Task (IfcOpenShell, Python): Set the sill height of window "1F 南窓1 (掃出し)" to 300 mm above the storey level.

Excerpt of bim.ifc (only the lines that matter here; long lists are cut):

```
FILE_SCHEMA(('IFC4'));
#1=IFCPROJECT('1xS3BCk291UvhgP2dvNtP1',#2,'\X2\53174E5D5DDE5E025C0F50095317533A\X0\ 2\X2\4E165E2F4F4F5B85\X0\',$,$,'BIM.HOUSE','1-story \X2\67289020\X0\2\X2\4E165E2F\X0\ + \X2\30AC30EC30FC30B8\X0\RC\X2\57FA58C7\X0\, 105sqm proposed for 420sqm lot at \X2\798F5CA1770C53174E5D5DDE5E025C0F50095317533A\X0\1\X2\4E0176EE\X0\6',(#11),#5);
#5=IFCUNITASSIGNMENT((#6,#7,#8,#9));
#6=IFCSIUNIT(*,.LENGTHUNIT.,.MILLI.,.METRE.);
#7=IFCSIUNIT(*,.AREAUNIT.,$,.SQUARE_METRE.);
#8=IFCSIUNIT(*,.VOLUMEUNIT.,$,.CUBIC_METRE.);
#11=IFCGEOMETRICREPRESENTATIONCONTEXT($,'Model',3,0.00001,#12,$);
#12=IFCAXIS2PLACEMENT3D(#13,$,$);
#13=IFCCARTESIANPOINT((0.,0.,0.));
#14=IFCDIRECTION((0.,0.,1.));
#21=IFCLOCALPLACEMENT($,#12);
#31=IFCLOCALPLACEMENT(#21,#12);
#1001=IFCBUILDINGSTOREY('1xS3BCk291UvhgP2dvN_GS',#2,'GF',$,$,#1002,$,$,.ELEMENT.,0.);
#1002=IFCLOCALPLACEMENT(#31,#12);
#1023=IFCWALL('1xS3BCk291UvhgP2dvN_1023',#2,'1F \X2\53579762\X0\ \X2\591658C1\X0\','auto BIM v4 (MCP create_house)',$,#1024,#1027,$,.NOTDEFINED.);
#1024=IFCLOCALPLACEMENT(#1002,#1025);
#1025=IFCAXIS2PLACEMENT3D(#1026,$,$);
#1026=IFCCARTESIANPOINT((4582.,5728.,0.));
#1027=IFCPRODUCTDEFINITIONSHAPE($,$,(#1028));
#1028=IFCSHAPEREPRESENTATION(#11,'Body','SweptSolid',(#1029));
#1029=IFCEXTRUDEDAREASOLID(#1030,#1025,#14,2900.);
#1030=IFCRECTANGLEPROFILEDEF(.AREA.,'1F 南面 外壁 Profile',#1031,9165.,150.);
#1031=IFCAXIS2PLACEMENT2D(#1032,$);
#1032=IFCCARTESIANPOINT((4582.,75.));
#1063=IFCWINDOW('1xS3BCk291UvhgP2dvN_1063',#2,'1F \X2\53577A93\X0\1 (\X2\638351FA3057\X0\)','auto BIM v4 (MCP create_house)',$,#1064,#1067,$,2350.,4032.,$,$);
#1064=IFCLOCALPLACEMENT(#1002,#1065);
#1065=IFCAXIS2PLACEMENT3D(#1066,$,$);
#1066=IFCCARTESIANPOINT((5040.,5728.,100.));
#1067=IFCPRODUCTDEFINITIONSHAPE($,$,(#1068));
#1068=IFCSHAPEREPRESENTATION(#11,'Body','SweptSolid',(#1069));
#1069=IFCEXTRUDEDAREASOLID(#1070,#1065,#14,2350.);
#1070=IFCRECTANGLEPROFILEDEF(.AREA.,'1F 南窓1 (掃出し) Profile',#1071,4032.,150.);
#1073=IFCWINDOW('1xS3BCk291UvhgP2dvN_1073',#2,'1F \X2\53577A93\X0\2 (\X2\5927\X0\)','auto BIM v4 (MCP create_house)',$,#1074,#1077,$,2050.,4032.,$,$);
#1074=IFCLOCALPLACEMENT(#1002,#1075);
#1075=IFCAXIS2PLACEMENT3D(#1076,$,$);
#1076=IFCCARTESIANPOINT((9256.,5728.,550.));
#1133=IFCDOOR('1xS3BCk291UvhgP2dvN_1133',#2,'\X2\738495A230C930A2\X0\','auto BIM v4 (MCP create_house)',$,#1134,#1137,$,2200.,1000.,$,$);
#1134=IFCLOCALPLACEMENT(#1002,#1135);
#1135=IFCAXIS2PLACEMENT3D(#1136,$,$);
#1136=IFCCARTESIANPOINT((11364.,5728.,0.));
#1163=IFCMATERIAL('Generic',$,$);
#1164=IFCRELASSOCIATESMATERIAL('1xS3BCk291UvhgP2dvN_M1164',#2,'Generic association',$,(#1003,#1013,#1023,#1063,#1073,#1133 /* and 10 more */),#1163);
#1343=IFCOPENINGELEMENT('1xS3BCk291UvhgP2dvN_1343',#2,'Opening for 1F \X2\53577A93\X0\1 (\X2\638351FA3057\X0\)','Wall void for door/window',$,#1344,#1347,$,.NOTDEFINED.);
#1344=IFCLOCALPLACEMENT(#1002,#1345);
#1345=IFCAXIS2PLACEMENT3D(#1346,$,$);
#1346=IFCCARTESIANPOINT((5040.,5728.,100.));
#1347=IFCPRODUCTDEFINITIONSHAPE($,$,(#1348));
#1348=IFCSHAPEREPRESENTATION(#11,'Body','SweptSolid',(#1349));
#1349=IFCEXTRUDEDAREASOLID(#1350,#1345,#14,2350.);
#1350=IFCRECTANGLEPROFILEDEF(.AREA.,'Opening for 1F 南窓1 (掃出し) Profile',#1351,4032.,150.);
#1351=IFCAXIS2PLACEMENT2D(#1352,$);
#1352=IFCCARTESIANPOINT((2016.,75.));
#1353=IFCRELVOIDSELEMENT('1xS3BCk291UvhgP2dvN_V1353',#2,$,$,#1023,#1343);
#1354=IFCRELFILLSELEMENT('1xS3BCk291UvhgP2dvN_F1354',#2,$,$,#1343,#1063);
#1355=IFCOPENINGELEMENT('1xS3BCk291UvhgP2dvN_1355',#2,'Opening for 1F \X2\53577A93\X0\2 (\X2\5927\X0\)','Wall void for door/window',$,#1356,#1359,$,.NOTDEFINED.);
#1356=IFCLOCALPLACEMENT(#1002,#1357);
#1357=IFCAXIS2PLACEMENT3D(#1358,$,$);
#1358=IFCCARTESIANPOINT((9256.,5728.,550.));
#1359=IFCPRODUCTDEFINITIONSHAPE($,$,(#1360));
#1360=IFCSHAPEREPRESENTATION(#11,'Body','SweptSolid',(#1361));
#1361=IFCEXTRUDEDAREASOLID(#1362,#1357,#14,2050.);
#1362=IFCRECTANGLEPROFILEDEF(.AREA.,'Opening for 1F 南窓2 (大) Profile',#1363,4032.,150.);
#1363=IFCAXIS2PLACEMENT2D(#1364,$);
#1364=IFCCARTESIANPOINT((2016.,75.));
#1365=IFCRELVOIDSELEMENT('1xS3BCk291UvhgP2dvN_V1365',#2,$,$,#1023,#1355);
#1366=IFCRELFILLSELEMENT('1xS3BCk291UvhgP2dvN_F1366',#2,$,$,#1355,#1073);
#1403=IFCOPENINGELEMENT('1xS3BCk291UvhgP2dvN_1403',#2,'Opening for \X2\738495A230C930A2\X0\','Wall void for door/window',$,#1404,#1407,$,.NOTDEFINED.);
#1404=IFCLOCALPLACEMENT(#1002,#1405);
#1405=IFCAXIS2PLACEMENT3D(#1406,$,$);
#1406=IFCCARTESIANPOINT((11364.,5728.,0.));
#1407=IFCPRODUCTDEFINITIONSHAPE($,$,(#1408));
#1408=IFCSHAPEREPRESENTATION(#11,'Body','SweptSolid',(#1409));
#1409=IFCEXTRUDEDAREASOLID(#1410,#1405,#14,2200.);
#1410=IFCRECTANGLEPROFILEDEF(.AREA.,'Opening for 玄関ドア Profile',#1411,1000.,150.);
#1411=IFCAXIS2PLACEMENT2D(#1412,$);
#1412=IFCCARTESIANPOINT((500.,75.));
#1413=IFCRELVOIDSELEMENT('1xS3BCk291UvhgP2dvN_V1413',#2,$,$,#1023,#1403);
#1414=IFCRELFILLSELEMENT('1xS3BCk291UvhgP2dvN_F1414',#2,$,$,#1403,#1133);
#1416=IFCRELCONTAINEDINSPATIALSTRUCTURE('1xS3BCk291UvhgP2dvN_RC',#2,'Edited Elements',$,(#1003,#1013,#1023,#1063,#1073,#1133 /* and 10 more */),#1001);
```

```python
import numpy as np
import ifcopenshell
import ifcopenshell.api.geometry
import ifcopenshell.geom
import ifcopenshell.util.element
import ifcopenshell.util.placement
import ifcopenshell.util.shape
import ifcopenshell.util.unit

model = ifcopenshell.open("bim.ifc")
unit_scale = ifcopenshell.util.unit.calculate_unit_scale(model)

window = model.by_guid("1xS3BCk291UvhgP2dvN_1063")
opening = window.FillsVoids[0].RelatingOpeningElement
storey = ifcopenshell.util.element.get_container(window, ifc_class="IfcBuildingStorey")
level = ifcopenshell.util.placement.get_local_placement(storey.ObjectPlacement)[2, 3]

# The opening's origin need not be at the sill, so measure its lowest point.
shape = ifcopenshell.geom.create_shape(ifcopenshell.geom.settings(), opening)
bottom = ifcopenshell.util.shape.get_shape_bottom_elevation(shape, shape.geometry) / unit_scale
dz = level + 0.3 / unit_scale - bottom

shift = np.array([0.0, 0.0, dz])
# The window is not placed relative to its opening, so move both.
for product in (opening, window):
    matrix = ifcopenshell.util.placement.get_local_placement(product.ObjectPlacement)
    matrix[:3, 3] += shift
    ifcopenshell.api.geometry.edit_object_placement(model, product=product, matrix=matrix, is_si=False)

print(f"moved by {dz * unit_scale:+.3f} m")

model.write("bim_v2.ifc")
```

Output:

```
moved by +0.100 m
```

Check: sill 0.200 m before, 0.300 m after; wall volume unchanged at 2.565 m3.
